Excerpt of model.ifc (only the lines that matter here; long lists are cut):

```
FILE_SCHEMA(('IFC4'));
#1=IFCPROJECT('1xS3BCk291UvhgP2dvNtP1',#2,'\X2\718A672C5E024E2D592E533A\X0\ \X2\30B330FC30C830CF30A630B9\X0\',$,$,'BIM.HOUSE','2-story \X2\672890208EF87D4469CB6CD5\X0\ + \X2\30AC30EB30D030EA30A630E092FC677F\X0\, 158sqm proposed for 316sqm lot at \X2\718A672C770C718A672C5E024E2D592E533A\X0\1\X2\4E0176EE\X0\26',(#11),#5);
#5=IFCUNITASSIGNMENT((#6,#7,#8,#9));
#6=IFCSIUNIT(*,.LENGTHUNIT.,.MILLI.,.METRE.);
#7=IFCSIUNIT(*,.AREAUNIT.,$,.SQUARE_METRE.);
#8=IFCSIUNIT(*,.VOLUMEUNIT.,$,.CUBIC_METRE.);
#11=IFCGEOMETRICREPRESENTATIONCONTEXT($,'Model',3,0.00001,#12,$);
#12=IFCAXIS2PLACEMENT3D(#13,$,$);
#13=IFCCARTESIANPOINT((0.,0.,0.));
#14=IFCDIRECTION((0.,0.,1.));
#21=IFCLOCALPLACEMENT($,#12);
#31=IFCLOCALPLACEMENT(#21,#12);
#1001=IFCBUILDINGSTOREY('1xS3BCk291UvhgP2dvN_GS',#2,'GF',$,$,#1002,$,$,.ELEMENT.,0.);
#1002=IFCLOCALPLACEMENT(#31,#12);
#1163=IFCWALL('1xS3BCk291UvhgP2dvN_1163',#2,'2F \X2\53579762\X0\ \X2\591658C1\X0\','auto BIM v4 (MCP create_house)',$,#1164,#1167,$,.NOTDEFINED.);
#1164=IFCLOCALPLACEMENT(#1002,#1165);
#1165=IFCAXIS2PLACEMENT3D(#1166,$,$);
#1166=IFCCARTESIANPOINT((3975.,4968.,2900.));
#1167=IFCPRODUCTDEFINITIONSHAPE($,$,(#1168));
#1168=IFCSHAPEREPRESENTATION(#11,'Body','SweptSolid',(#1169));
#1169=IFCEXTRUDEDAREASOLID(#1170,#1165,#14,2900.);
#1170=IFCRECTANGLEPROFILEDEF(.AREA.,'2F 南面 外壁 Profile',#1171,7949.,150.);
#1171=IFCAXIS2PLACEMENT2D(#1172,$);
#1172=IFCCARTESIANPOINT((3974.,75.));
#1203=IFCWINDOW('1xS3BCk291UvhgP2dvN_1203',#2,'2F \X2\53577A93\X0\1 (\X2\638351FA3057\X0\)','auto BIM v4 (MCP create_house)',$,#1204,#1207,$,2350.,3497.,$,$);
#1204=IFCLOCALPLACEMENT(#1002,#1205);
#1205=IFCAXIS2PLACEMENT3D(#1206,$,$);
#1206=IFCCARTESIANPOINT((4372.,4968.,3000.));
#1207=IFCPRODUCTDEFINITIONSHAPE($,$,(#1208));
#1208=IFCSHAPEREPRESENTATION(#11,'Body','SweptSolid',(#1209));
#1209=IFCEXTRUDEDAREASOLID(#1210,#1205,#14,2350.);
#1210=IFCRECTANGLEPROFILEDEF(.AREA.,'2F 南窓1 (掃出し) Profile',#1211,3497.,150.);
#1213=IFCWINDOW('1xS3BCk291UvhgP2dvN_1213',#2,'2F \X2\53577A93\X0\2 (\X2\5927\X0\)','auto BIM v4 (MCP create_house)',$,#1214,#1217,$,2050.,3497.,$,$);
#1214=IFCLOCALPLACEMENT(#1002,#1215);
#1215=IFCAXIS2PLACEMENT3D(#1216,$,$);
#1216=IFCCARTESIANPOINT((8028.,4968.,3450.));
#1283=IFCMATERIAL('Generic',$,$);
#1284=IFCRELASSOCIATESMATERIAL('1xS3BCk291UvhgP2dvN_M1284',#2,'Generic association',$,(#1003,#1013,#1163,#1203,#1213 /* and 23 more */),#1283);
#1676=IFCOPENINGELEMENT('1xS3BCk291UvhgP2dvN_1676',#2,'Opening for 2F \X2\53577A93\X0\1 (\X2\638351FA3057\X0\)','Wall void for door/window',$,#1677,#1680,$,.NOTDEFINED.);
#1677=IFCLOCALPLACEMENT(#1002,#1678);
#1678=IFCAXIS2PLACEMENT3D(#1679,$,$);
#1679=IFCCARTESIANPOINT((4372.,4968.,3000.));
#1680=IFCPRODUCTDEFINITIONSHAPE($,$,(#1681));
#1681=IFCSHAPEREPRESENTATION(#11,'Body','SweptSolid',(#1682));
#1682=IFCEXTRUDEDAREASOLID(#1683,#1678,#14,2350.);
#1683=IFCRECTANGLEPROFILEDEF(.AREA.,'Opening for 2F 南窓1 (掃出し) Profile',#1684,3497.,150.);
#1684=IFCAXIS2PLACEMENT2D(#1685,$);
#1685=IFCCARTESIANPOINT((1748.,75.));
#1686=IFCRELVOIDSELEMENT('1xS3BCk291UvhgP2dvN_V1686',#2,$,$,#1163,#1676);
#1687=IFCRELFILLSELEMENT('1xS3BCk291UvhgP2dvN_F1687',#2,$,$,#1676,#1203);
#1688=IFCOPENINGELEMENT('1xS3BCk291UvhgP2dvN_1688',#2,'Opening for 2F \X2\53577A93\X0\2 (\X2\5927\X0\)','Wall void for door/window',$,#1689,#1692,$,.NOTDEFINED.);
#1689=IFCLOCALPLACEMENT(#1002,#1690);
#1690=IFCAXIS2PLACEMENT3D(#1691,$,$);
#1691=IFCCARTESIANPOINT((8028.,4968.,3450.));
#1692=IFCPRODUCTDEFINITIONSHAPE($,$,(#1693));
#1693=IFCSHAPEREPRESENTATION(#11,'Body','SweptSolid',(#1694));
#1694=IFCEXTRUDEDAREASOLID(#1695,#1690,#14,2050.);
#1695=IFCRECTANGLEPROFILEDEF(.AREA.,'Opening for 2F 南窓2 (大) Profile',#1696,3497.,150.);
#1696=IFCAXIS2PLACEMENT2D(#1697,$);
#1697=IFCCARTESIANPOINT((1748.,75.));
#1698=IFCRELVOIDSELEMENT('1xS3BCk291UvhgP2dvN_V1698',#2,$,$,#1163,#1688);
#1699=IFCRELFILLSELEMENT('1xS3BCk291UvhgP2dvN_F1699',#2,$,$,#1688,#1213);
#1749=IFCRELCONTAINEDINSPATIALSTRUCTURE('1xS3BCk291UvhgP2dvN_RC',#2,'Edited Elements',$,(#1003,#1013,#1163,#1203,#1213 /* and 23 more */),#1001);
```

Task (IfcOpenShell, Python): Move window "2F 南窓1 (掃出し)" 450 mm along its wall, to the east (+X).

```python
import ifcopenshell
import ifcopenshell.api.geometry
import ifcopenshell.util.placement

model = ifcopenshell.open("model.ifc")

window = model.by_id(1203)
opening = window.FillsVoids[0].RelatingOpeningElement
wall = opening.VoidsElements[0].RelatingBuildingElement

wall_matrix = ifcopenshell.util.placement.get_local_placement(wall.ObjectPlacement)
shift = wall_matrix[:3, 0] * 450.0
before = ifcopenshell.util.placement.get_local_placement(window.ObjectPlacement)[:3, 3].copy()

# The window is not placed relative to its opening, so move both.
for product in (opening, window):
    matrix = ifcopenshell.util.placement.get_local_placement(product.ObjectPlacement)
    matrix[:3, 3] += shift
    ifcopenshell.api.geometry.edit_object_placement(model, product=product, matrix=matrix, is_si=False)

after = ifcopenshell.util.placement.get_local_placement(window.ObjectPlacement)[:3, 3]
print("window moved by", (after - before).round(3) + 0.0)

model.write("model_v2.ifc")
```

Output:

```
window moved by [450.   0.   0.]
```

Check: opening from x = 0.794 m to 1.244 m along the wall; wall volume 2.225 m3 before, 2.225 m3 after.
